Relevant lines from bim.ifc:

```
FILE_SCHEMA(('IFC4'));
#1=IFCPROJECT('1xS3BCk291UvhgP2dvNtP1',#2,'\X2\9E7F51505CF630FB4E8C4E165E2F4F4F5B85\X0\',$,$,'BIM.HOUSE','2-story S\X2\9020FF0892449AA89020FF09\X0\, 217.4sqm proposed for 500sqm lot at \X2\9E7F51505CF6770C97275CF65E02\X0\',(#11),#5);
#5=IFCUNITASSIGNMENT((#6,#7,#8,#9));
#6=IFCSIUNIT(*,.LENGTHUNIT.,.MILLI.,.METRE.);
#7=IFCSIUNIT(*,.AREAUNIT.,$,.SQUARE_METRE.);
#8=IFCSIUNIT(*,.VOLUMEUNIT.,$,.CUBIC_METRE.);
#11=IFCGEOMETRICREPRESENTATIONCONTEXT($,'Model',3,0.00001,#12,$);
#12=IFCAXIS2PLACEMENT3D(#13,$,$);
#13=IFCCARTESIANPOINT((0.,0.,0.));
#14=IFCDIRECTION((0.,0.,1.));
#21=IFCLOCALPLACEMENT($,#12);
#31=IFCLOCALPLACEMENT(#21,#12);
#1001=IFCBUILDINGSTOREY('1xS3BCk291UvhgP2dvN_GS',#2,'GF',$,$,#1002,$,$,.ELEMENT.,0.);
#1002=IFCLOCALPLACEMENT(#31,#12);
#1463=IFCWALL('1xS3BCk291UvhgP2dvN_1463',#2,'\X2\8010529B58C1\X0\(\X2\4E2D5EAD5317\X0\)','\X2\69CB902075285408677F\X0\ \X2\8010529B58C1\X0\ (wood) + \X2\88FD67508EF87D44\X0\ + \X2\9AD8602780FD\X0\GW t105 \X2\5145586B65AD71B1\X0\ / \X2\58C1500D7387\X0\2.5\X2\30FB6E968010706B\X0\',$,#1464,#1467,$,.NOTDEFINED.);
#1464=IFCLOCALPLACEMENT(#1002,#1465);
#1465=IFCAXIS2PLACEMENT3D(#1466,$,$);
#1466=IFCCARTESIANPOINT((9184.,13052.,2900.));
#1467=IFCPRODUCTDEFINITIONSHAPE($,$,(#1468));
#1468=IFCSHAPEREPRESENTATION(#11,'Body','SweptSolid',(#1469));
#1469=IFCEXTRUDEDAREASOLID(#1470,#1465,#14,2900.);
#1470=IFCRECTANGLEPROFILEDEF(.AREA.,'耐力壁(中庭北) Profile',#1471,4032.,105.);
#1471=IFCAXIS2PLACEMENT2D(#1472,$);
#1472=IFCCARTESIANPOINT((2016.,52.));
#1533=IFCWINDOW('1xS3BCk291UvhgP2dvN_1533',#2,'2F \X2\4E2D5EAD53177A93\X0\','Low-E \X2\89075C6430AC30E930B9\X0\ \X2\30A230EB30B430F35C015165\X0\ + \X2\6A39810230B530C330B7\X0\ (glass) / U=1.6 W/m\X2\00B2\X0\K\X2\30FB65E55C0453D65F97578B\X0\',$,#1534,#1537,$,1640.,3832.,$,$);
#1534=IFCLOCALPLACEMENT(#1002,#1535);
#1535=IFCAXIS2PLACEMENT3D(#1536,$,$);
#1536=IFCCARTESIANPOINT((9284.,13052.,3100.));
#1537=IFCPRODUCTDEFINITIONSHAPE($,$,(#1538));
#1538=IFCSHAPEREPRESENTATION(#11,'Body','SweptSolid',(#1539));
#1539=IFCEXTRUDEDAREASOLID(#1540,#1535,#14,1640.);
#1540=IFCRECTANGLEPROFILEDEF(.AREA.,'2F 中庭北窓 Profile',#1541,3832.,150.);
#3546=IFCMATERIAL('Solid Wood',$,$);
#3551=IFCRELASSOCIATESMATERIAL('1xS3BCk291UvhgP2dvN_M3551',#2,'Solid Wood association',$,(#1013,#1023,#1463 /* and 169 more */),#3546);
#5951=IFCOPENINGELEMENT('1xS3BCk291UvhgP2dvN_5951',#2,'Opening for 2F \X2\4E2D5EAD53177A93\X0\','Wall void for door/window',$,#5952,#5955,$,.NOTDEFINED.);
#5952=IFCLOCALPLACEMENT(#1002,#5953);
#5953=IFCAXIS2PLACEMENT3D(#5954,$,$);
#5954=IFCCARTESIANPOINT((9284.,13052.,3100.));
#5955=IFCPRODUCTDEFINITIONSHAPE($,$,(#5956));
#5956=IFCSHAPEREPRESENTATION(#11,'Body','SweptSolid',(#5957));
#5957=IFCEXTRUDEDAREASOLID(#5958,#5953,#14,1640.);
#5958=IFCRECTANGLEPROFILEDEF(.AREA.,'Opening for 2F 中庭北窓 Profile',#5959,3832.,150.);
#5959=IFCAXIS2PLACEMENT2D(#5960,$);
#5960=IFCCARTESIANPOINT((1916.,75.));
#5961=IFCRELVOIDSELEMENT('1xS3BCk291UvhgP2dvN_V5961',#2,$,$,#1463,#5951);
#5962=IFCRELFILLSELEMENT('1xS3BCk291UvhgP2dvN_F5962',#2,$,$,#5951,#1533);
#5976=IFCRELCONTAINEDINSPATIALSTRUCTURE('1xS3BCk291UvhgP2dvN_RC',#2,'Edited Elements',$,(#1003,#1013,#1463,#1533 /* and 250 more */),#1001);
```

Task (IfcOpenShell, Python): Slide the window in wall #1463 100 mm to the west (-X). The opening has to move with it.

```python
import ifcopenshell
import ifcopenshell.api.geometry
import ifcopenshell.util.placement

model = ifcopenshell.open("bim.ifc")

window = model.by_guid("1xS3BCk291UvhgP2dvN_1533")
opening = window.FillsVoids[0].RelatingOpeningElement
wall = opening.VoidsElements[0].RelatingBuildingElement

wall_matrix = ifcopenshell.util.placement.get_local_placement(wall.ObjectPlacement)
shift = wall_matrix[:3, 0] * -100.0
before = ifcopenshell.util.placement.get_local_placement(window.ObjectPlacement)[:3, 3].copy()

# The window is not placed relative to its opening, so move both.
for product in (opening, window):
    matrix = ifcopenshell.util.placement.get_local_placement(product.ObjectPlacement)
    matrix[:3, 3] += shift
    ifcopenshell.api.geometry.edit_object_placement(model, product=product, matrix=matrix, is_si=False)

after = ifcopenshell.util.placement.get_local_placement(window.ObjectPlacement)[:3, 3]
print("window moved by", (after - before).round(3) + 0.0)

model.write("bim-out.ifc")
```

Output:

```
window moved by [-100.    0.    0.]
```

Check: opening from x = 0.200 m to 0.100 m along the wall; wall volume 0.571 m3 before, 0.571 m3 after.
